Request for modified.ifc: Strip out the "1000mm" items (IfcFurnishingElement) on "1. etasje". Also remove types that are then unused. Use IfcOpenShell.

First a look at what the model holds.

```python
import ifcopenshell
import ifcopenshell.util.element

model = ifcopenshell.open("modified.ifc")
print(model.schema)
storey = next(s for s in model.by_type("IfcBuildingStorey") if s.Name == "1. etasje")
furniture = [e for e in ifcopenshell.util.element.get_decomposition(storey) if e.is_a("IfcFurnishingElement")]
seen = {}
for e in furniture:
    element_type = ifcopenshell.util.element.get_type(e)
    name = element_type.Name if element_type not in (None, e) else None
    seen[name] = seen.get(name, 0) + 1
for name, count in sorted(seen.items(), key=str):
    print(count, "x", name)
```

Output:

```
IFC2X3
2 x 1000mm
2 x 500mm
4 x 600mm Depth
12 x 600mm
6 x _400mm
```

```python
import ifcopenshell
import ifcopenshell.api.root
import ifcopenshell.util.element

model = ifcopenshell.open("modified.ifc")

storey = next(s for s in model.by_type("IfcBuildingStorey") if s.Name == "1. etasje")
furniture = [e for e in ifcopenshell.util.element.get_decomposition(storey) if e.is_a("IfcFurnishingElement")]
targets = [e for e in furniture if (t := ifcopenshell.util.element.get_type(e)) not in (None, e) and t.Name == "1000mm"]
types = {ifcopenshell.util.element.get_type(e) for e in targets} - {None, *targets}

for e in targets:
    ifcopenshell.api.root.remove_product(model, product=e)
print(len(targets), "removed")

unused = [t for t in types if not ifcopenshell.util.element.get_types(t)]
for t in unused:
    ifcopenshell.api.root.remove_product(model, product=t)
print(len(unused), "unused types removed")

model.write("modified_edited.ifc")
```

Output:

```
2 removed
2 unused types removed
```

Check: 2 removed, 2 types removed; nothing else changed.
